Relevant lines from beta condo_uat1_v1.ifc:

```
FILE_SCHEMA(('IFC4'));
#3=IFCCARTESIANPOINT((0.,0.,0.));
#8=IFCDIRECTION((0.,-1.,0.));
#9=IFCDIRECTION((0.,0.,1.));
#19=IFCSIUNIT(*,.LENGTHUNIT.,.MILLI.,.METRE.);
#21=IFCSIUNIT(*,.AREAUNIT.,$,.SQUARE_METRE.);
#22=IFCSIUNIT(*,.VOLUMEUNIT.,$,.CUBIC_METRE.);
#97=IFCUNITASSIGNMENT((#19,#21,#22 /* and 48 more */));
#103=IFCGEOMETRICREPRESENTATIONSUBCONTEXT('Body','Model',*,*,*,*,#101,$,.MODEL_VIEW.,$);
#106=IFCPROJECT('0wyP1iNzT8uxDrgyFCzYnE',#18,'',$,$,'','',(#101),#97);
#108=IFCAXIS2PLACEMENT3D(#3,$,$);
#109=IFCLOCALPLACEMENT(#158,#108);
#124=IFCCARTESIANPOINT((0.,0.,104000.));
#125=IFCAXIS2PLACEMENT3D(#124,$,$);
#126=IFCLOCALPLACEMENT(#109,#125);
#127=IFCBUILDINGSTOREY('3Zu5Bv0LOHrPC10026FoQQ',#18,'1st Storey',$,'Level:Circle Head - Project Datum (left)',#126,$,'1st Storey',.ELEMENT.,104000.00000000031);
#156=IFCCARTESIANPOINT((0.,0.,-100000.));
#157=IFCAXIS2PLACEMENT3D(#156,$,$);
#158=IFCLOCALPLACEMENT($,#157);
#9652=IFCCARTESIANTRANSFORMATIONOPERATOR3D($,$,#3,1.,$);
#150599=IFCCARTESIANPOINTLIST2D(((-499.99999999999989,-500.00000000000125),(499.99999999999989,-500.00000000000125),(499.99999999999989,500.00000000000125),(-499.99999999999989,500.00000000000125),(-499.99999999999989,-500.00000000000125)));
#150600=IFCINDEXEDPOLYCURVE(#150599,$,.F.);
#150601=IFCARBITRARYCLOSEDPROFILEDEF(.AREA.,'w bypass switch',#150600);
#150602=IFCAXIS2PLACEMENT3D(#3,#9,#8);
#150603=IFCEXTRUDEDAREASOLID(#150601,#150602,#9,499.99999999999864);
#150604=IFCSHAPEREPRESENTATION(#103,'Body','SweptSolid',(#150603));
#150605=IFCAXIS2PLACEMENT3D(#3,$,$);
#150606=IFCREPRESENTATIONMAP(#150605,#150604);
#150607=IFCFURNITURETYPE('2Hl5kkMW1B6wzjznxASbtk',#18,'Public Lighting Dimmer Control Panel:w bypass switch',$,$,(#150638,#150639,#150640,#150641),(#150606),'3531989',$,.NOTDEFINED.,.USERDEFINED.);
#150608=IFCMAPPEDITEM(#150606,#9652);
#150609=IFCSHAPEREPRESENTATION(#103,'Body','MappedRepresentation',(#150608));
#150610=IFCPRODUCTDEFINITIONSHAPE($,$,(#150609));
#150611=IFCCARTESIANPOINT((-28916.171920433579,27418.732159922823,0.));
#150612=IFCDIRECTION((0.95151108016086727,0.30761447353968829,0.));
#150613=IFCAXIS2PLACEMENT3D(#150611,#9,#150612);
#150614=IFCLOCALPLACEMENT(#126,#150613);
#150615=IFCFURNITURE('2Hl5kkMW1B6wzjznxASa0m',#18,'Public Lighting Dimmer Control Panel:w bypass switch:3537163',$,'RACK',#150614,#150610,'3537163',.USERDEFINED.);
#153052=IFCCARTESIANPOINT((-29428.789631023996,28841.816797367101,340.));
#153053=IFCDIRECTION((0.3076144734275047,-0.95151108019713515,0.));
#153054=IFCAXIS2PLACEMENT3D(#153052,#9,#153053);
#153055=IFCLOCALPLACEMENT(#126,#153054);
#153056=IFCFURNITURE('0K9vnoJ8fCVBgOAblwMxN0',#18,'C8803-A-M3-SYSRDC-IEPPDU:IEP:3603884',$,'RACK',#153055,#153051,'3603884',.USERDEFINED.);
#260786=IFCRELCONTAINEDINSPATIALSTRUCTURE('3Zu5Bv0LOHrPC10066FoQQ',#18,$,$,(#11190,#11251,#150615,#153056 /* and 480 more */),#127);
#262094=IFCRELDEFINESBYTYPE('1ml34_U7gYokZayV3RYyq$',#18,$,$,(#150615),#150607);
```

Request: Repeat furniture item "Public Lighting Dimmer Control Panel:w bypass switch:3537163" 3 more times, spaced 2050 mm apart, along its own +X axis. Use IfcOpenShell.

```python
import ifcopenshell
import ifcopenshell.api.geometry
import ifcopenshell.api.root
import ifcopenshell.util.element
import ifcopenshell.util.placement
import ifcopenshell.util.unit

model = ifcopenshell.open("beta condo_uat1_v1.ifc")
unit_scale = ifcopenshell.util.unit.calculate_unit_scale(model)


def reuse_history(source, copy):
    """copy_class also copies each property set's owner history, people and application; keep the originals."""
    for rel in copy.IsDefinedBy:
        if rel.is_a("IfcRelDefinesByProperties") and (history := rel.RelatingPropertyDefinition.OwnerHistory):
            rel.RelatingPropertyDefinition.OwnerHistory = source.OwnerHistory
            ifcopenshell.util.element.remove_deep2(model, history)


source = model.by_guid("2Hl5kkMW1B6wzjznxASa0m")
base = ifcopenshell.util.placement.get_local_placement(source.ObjectPlacement)
step = base[:3, 0] * 2.05 / unit_scale

for i in range(1, 4):
    copy = ifcopenshell.api.root.copy_class(model, product=source)
    copy.Representation = ifcopenshell.util.element.copy_deep(
        model, source.Representation, exclude=["IfcGeometricRepresentationContext", "IfcRepresentationMap"]
    )
    copy.Name = "Public Lighting Dimmer Control Panel:w bypass switch"
    copy.Tag = None
    reuse_history(source, copy)
    matrix = base.copy()
    matrix[:3, 3] += i * step
    print("added at", matrix[:3, 3].round(3) + 0.0)
    ifcopenshell.api.geometry.edit_object_placement(model, product=copy, matrix=matrix, is_si=False)

model.write("beta condo_uat1_v1_edited.ifc")
```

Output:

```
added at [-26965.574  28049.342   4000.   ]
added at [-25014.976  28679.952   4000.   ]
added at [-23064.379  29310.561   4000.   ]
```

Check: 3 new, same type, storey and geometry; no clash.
